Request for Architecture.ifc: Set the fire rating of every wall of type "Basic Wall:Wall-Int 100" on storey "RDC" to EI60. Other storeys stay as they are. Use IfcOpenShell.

First a look at what the model holds.

```python
import ifcopenshell
import ifcopenshell.util.element

model = ifcopenshell.open("Architecture.ifc")
print(model.schema)
storey = next(s for s in model.by_type("IfcBuildingStorey") if s.Name == "RDC")
walls = [e for e in ifcopenshell.util.element.get_decomposition(storey) if e.is_a("IfcWall")]
seen = {}
for e in walls:
    element_type = ifcopenshell.util.element.get_type(e)
    key = (element_type.Name if element_type != e and element_type else None, ifcopenshell.util.element.get_pset(e, "Pset_WallCommon", "FireRating"))
    seen[key] = seen.get(key, 0) + 1
for (name, value), count in sorted(seen.items(), key=str):
    print(count, "x", name, "|", value)
```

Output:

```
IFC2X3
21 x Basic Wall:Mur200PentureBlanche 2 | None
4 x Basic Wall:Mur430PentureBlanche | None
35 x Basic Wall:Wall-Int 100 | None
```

```python
import ifcopenshell
import ifcopenshell.api.pset
import ifcopenshell.util.element

model = ifcopenshell.open("Architecture.ifc")

storey = next(s for s in model.by_type("IfcBuildingStorey") if s.Name == "RDC")
walls = [e for e in ifcopenshell.util.element.get_decomposition(storey) if e.is_a("IfcWall")]

count = 0
for e in walls:
    element_type = ifcopenshell.util.element.get_type(e)
    if element_type in (None, e) or element_type.Name != "Basic Wall:Wall-Int 100":
        continue
    # add_pset returns the element's existing set when there is one.
    pset = ifcopenshell.api.pset.add_pset(model, product=e, name="Pset_WallCommon")
    ifcopenshell.api.pset.edit_pset(model, pset=pset, properties={"FireRating": "EI60"})
    count += 1

print(count, "walls updated")

model.write("Architecture-out.ifc")
```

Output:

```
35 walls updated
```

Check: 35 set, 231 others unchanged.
